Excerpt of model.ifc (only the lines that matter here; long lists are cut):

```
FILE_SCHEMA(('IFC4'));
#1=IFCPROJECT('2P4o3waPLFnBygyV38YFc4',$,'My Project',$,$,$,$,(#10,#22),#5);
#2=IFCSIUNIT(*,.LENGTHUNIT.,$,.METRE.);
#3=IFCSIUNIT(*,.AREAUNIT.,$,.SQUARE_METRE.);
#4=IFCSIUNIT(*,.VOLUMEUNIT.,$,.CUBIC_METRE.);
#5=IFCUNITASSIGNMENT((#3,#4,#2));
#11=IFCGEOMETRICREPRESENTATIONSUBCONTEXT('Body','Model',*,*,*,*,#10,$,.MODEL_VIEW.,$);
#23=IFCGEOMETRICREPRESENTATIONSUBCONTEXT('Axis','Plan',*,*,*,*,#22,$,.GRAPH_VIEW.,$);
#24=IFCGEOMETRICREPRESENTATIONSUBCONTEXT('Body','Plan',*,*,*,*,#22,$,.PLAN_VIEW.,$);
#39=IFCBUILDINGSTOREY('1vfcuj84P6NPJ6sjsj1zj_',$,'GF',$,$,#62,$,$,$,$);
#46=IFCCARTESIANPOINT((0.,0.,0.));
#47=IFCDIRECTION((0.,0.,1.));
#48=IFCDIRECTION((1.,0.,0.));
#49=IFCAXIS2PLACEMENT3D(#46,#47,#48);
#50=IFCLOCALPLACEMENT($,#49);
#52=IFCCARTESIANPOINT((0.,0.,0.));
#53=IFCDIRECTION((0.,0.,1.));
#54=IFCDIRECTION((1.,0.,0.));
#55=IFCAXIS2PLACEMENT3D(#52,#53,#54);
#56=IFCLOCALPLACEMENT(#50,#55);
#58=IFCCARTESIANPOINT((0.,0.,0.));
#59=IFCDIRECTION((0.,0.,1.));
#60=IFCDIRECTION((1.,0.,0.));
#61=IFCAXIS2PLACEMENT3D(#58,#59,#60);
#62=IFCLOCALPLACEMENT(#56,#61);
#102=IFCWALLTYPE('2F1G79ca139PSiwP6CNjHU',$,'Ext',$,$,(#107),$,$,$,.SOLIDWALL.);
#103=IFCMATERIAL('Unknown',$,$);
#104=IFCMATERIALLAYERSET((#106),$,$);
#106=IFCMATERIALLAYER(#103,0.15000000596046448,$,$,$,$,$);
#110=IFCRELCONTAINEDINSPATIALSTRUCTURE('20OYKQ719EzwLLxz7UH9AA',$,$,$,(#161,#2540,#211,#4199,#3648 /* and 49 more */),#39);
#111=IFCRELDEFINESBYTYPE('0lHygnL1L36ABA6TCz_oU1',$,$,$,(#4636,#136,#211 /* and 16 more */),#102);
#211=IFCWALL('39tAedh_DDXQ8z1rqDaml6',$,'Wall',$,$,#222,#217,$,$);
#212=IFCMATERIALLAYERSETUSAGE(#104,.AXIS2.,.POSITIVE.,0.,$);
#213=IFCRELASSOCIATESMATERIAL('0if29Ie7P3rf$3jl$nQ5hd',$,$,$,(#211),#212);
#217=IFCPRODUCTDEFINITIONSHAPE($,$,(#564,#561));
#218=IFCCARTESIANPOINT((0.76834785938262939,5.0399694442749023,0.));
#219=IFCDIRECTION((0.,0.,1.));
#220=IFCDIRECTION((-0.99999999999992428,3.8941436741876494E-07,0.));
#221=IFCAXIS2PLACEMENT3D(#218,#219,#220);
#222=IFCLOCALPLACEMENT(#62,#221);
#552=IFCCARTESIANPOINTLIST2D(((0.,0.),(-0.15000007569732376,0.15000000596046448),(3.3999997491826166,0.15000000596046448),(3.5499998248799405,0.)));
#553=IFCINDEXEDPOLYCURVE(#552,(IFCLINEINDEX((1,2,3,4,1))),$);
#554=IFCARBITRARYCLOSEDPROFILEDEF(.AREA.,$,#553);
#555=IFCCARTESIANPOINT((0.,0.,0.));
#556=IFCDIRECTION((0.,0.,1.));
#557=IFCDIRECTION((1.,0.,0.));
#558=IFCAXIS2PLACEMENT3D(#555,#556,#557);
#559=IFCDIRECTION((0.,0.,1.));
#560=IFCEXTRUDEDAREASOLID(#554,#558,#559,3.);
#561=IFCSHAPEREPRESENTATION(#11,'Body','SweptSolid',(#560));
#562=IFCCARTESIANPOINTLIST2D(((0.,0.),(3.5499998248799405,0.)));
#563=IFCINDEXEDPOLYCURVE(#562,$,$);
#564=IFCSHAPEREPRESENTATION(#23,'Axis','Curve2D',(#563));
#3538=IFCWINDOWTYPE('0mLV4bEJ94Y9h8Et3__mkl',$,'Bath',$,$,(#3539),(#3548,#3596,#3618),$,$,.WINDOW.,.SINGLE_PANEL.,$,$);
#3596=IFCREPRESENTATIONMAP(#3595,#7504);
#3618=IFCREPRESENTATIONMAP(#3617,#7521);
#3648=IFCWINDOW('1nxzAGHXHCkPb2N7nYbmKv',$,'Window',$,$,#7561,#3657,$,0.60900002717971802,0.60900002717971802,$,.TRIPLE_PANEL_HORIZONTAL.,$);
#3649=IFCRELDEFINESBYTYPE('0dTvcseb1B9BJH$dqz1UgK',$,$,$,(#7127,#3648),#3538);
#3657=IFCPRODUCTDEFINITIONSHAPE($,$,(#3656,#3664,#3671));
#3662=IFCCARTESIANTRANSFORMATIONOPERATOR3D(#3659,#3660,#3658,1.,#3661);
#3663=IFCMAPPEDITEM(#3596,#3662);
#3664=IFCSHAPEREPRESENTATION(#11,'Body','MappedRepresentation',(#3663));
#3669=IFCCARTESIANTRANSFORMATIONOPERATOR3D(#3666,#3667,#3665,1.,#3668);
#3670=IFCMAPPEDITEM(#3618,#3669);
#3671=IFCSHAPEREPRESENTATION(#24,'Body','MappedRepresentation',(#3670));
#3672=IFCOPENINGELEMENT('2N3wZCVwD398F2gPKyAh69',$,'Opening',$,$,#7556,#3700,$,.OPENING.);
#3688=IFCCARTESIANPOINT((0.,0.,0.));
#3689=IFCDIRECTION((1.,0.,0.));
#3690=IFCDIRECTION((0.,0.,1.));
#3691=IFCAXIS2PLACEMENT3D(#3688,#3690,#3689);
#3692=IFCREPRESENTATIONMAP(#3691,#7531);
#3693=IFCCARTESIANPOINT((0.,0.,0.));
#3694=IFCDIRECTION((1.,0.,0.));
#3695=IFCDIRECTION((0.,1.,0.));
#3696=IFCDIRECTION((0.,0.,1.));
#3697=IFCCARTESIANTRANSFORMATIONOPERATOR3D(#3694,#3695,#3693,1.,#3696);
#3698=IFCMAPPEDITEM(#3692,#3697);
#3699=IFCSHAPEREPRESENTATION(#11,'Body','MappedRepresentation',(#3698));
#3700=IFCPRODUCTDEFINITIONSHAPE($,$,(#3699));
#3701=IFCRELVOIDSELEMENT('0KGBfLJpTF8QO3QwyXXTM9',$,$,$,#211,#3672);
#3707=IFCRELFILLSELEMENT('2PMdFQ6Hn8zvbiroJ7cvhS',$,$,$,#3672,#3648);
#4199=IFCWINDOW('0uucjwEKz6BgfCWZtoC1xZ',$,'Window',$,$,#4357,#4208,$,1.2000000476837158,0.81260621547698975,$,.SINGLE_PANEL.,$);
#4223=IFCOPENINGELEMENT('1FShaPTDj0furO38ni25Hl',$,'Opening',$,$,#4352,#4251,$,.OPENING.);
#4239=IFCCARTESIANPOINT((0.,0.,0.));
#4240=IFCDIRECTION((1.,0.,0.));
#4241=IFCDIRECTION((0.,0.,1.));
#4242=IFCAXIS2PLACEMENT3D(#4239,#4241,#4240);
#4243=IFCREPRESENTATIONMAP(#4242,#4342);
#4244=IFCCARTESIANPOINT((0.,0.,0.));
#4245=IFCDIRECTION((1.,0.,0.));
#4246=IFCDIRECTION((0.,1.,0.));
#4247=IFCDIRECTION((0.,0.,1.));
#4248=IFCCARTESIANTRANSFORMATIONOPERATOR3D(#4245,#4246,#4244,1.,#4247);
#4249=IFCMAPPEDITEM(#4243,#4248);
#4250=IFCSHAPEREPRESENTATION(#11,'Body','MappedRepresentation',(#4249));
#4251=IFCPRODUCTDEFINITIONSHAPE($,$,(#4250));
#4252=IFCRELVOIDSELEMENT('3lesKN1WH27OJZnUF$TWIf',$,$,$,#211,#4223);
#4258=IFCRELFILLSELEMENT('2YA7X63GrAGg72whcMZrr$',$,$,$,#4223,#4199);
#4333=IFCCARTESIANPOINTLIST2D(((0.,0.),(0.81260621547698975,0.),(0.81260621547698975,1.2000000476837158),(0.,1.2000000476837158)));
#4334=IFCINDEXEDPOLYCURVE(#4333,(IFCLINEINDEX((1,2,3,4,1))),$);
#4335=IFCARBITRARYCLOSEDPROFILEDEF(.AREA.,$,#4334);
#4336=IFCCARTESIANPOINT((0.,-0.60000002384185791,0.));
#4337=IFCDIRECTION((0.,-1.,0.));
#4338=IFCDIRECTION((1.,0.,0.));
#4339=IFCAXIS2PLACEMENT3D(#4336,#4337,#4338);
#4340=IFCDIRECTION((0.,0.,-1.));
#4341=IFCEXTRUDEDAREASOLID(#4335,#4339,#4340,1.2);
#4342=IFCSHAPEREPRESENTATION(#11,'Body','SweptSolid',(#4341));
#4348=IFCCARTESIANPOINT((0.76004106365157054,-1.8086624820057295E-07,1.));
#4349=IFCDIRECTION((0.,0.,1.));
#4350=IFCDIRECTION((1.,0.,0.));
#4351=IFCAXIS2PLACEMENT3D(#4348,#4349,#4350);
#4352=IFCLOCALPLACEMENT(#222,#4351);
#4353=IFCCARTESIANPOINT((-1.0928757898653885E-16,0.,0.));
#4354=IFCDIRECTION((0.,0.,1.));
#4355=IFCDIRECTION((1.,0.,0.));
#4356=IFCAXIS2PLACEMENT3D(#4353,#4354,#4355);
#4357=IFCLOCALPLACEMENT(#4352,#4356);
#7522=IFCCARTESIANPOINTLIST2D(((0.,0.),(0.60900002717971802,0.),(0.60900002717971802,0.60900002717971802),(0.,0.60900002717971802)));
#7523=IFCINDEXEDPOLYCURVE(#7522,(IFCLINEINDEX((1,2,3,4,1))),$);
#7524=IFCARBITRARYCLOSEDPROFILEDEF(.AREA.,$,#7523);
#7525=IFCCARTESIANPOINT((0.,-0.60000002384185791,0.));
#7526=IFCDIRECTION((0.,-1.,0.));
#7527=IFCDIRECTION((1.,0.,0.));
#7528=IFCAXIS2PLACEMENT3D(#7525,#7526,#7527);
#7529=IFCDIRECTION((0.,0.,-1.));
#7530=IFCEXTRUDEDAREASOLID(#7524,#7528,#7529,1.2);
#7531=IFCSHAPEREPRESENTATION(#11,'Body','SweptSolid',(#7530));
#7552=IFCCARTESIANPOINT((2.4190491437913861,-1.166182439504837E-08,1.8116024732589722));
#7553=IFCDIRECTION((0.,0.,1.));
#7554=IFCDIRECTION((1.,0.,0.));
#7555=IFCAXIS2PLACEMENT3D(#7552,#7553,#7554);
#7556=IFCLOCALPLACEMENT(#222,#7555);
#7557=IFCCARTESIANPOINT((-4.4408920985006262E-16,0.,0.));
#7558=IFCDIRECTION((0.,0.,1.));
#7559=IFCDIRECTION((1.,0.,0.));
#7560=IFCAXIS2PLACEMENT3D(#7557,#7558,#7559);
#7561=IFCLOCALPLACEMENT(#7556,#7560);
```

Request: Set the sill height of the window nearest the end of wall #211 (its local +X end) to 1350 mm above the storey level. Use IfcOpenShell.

```python
import numpy as np
import ifcopenshell
import ifcopenshell.api.geometry
import ifcopenshell.geom
import ifcopenshell.util.element
import ifcopenshell.util.placement
import ifcopenshell.util.shape
import ifcopenshell.util.unit

model = ifcopenshell.open("model.ifc")
unit_scale = ifcopenshell.util.unit.calculate_unit_scale(model)

window = model.by_id(3648)
opening = window.FillsVoids[0].RelatingOpeningElement
storey = ifcopenshell.util.element.get_container(window, ifc_class="IfcBuildingStorey")
level = ifcopenshell.util.placement.get_local_placement(storey.ObjectPlacement)[2, 3]

# The opening's origin need not be at the sill, so measure its lowest point.
shape = ifcopenshell.geom.create_shape(ifcopenshell.geom.settings(), opening)
bottom = ifcopenshell.util.shape.get_shape_bottom_elevation(shape, shape.geometry) / unit_scale
dz = level + 1.35 / unit_scale - bottom

shift = np.array([0.0, 0.0, dz])
# The window is placed relative to its opening, so it follows when the opening moves.
matrix = ifcopenshell.util.placement.get_local_placement(opening.ObjectPlacement)
matrix[:3, 3] += shift
ifcopenshell.api.geometry.edit_object_placement(
    model, product=opening, matrix=matrix, is_si=False, should_transform_children=True
)

print(f"moved by {dz * unit_scale:+.3f} m")

model.write("model_rev.ifc")
```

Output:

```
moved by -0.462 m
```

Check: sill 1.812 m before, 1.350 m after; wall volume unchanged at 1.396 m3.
